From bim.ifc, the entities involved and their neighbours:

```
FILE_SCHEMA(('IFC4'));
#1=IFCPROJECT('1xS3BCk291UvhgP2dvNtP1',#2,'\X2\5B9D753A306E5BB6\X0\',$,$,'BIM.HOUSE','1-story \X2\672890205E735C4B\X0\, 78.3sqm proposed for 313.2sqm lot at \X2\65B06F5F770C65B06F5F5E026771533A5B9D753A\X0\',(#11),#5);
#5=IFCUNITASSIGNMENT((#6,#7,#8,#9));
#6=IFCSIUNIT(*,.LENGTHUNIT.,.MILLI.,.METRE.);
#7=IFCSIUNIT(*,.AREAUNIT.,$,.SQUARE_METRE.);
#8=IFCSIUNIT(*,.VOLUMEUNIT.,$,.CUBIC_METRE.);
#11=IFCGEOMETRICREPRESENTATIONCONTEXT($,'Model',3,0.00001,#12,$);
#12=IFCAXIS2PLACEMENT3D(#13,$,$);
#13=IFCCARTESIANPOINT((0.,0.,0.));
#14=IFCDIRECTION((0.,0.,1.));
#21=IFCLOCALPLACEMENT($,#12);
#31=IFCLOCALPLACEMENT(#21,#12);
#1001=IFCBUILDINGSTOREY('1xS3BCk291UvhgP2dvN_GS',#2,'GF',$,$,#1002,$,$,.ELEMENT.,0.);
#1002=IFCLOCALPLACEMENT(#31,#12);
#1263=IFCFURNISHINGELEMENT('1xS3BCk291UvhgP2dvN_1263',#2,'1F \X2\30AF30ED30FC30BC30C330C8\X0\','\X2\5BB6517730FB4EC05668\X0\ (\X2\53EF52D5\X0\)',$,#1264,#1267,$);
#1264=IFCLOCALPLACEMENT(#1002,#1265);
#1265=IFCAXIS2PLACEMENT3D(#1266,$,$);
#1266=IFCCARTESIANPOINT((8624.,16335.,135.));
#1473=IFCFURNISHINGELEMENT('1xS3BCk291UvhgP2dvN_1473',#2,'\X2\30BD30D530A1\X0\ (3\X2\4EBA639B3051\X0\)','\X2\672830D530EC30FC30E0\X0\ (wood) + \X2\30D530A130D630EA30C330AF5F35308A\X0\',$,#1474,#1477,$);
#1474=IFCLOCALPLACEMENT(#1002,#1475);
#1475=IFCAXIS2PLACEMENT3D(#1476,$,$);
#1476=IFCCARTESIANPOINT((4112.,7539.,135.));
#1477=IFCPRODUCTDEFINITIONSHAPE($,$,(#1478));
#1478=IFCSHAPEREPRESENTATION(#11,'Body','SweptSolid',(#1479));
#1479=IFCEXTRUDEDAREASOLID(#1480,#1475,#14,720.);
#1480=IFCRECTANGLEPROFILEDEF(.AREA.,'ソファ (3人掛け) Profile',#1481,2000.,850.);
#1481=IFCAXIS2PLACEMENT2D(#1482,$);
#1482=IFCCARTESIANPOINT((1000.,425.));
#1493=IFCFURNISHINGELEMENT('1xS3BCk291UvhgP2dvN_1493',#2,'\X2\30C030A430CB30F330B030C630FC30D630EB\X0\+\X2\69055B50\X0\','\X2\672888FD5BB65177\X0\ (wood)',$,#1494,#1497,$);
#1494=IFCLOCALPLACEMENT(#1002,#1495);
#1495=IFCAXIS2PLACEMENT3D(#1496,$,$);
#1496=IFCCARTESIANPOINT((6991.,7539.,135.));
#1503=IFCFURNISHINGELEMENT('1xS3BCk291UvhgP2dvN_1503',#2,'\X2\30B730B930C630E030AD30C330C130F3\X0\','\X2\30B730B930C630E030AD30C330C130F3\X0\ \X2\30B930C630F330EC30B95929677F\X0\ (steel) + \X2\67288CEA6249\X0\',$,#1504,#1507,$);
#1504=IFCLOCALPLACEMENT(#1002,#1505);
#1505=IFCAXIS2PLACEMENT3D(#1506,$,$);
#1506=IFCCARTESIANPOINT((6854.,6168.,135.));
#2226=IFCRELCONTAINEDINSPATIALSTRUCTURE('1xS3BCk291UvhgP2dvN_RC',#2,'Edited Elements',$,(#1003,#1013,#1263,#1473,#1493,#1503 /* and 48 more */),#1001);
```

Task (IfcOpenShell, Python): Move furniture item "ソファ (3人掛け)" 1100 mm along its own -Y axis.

```python
import ifcopenshell
import ifcopenshell.api.geometry
import ifcopenshell.util.placement

model = ifcopenshell.open("bim.ifc")

item = model.by_guid("1xS3BCk291UvhgP2dvN_1473")
matrix = ifcopenshell.util.placement.get_local_placement(item.ObjectPlacement)
matrix[:3, 3] -= matrix[:3, 1] * 1100.0
ifcopenshell.api.geometry.edit_object_placement(model, product=item, matrix=matrix, is_si=False)

print(ifcopenshell.util.placement.get_local_placement(item.ObjectPlacement).round(3) + 0.0)

model.write("bim_rev.ifc")
```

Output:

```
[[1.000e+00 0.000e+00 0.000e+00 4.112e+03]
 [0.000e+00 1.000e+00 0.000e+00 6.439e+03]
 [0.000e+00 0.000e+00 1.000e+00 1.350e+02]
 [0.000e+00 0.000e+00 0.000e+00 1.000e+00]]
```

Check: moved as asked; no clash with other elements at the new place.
